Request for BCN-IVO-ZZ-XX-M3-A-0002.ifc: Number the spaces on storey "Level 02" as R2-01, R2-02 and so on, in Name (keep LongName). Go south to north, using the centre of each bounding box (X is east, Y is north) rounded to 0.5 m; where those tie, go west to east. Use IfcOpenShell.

First a look at what the model holds.

```python
import ifcopenshell
import ifcopenshell.util.element
import ifcopenshell.util.placement

model = ifcopenshell.open("BCN-IVO-ZZ-XX-M3-A-0002.ifc")
print(model.schema)
storey = next(s for s in model.by_type("IfcBuildingStorey") if s.Name == "Level 02")
spaces = [e for e in ifcopenshell.util.element.get_decomposition(storey) if e.is_a("IfcSpace")]
for e in sorted(spaces, key=lambda e: e.id()):
    origin = ifcopenshell.util.placement.get_local_placement(e.ObjectPlacement)[:3, 3]
    print(e.id(), e.Name, e.LongName, origin.round(2) + 0.0, sep=" | ")
```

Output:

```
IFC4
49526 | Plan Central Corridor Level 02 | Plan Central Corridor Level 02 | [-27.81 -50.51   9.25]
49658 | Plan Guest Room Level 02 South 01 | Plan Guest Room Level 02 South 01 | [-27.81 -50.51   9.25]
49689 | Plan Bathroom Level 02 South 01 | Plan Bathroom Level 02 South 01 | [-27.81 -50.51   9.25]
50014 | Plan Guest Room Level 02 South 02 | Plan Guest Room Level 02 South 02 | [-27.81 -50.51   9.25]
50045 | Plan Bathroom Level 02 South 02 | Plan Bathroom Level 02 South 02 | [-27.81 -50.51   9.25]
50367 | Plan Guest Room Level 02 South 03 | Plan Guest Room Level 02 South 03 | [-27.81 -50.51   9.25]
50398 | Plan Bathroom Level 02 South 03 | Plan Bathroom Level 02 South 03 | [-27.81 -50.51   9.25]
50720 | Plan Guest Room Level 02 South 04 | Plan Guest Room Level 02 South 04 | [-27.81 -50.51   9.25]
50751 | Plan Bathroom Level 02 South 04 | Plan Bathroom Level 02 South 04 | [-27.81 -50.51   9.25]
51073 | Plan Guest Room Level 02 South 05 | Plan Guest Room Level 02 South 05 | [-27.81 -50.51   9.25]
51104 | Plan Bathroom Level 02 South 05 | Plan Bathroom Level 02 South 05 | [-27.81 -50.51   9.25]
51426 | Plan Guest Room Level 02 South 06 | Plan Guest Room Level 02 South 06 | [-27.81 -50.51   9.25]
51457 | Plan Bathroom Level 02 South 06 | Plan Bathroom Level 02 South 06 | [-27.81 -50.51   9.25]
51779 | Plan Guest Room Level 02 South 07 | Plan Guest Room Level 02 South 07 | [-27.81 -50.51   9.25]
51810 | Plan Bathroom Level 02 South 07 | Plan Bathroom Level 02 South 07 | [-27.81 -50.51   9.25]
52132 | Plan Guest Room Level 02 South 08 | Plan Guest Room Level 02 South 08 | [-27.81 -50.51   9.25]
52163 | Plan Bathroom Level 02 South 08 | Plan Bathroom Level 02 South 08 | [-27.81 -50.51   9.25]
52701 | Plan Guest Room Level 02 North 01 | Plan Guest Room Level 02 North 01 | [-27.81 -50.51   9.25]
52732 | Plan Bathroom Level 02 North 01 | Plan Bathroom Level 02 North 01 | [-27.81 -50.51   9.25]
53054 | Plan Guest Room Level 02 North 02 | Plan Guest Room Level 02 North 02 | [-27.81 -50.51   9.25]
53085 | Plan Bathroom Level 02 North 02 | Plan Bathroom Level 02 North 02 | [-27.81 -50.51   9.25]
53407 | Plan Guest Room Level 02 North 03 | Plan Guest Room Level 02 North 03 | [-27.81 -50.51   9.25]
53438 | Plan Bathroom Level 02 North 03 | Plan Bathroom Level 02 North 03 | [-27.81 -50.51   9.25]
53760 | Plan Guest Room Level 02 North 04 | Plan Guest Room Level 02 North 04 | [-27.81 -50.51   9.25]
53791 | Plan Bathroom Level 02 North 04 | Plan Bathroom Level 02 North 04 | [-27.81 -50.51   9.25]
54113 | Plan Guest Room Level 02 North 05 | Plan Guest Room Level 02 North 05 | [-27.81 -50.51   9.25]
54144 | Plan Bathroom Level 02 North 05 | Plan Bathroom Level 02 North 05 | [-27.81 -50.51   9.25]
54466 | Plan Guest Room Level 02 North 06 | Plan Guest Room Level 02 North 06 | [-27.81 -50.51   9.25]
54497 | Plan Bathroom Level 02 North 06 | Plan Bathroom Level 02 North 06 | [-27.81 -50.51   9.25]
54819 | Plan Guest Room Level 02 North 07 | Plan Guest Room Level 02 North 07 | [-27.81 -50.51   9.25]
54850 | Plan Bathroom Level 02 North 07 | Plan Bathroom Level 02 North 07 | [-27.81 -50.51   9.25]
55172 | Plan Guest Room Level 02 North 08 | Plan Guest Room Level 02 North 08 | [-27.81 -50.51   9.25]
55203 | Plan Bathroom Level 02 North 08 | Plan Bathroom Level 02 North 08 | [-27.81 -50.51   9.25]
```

```python
import ifcopenshell
import ifcopenshell.geom
import ifcopenshell.util.element
import ifcopenshell.util.shape

model = ifcopenshell.open("BCN-IVO-ZZ-XX-M3-A-0002.ifc")
settings = ifcopenshell.geom.settings()
settings.set("use-world-coords", True)


def centre(element):
    shape = ifcopenshell.geom.create_shape(settings, element)
    return ifcopenshell.util.shape.get_bbox_centroid(shape.geometry)


storey = next(s for s in model.by_type("IfcBuildingStorey") if s.Name == "Level 02")
spaces = [e for e in ifcopenshell.util.element.get_decomposition(storey) if e.is_a("IfcSpace")]

# Insertion points can sit at a corner or the storey origin, so sort by the geometry (in metres).
centres = {e: centre(e) for e in spaces}
spaces.sort(key=lambda e: (round(centres[e][1] / 0.5), centres[e][0]))

for i, e in enumerate(spaces, start=1):
    number = f"R2-{i:02d}"
    e.Name = number
    print(e.id(), number)

model.write("BCN-IVO-ZZ-XX-M3-A-0002-out.ifc")
```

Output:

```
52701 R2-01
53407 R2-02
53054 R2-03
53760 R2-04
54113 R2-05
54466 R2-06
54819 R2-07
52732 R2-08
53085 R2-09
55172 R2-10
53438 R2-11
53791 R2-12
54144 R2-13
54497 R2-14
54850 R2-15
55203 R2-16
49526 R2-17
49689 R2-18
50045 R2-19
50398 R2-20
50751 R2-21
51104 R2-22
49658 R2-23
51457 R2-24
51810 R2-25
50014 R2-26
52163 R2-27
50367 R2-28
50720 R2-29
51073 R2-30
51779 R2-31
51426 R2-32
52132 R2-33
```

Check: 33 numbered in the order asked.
